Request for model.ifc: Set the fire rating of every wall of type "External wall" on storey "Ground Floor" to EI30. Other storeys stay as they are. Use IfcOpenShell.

First a look at what the model holds.

```python
import ifcopenshell
import ifcopenshell.util.element

model = ifcopenshell.open("model.ifc")
print(model.schema)
storey = next(s for s in model.by_type("IfcBuildingStorey") if s.Name == "Ground Floor")
walls = [e for e in ifcopenshell.util.element.get_decomposition(storey) if e.is_a("IfcWall")]
seen = {}
for e in walls:
    element_type = ifcopenshell.util.element.get_type(e)
    key = (element_type.Name if element_type != e and element_type else None, ifcopenshell.util.element.get_pset(e, "Pset_WallCommon", "FireRating"))
    seen[key] = seen.get(key, 0) + 1
for (name, value), count in sorted(seen.items(), key=str):
    print(count, "x", name, "|", value)
```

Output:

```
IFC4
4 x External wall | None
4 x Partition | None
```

```python
import ifcopenshell
import ifcopenshell.api.pset
import ifcopenshell.util.element

model = ifcopenshell.open("model.ifc")

storey = next(s for s in model.by_type("IfcBuildingStorey") if s.Name == "Ground Floor")
walls = [e for e in ifcopenshell.util.element.get_decomposition(storey) if e.is_a("IfcWall")]

count = 0
for e in walls:
    element_type = ifcopenshell.util.element.get_type(e)
    if element_type in (None, e) or element_type.Name != "External wall":
        continue
    # add_pset returns the element's existing set when there is one.
    pset = ifcopenshell.api.pset.add_pset(model, product=e, name="Pset_WallCommon")
    ifcopenshell.api.pset.edit_pset(model, pset=pset, properties={"FireRating": "EI30"})
    count += 1

print(count, "walls updated")

model.write("model_updated.ifc")
```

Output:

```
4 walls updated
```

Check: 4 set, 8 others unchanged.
